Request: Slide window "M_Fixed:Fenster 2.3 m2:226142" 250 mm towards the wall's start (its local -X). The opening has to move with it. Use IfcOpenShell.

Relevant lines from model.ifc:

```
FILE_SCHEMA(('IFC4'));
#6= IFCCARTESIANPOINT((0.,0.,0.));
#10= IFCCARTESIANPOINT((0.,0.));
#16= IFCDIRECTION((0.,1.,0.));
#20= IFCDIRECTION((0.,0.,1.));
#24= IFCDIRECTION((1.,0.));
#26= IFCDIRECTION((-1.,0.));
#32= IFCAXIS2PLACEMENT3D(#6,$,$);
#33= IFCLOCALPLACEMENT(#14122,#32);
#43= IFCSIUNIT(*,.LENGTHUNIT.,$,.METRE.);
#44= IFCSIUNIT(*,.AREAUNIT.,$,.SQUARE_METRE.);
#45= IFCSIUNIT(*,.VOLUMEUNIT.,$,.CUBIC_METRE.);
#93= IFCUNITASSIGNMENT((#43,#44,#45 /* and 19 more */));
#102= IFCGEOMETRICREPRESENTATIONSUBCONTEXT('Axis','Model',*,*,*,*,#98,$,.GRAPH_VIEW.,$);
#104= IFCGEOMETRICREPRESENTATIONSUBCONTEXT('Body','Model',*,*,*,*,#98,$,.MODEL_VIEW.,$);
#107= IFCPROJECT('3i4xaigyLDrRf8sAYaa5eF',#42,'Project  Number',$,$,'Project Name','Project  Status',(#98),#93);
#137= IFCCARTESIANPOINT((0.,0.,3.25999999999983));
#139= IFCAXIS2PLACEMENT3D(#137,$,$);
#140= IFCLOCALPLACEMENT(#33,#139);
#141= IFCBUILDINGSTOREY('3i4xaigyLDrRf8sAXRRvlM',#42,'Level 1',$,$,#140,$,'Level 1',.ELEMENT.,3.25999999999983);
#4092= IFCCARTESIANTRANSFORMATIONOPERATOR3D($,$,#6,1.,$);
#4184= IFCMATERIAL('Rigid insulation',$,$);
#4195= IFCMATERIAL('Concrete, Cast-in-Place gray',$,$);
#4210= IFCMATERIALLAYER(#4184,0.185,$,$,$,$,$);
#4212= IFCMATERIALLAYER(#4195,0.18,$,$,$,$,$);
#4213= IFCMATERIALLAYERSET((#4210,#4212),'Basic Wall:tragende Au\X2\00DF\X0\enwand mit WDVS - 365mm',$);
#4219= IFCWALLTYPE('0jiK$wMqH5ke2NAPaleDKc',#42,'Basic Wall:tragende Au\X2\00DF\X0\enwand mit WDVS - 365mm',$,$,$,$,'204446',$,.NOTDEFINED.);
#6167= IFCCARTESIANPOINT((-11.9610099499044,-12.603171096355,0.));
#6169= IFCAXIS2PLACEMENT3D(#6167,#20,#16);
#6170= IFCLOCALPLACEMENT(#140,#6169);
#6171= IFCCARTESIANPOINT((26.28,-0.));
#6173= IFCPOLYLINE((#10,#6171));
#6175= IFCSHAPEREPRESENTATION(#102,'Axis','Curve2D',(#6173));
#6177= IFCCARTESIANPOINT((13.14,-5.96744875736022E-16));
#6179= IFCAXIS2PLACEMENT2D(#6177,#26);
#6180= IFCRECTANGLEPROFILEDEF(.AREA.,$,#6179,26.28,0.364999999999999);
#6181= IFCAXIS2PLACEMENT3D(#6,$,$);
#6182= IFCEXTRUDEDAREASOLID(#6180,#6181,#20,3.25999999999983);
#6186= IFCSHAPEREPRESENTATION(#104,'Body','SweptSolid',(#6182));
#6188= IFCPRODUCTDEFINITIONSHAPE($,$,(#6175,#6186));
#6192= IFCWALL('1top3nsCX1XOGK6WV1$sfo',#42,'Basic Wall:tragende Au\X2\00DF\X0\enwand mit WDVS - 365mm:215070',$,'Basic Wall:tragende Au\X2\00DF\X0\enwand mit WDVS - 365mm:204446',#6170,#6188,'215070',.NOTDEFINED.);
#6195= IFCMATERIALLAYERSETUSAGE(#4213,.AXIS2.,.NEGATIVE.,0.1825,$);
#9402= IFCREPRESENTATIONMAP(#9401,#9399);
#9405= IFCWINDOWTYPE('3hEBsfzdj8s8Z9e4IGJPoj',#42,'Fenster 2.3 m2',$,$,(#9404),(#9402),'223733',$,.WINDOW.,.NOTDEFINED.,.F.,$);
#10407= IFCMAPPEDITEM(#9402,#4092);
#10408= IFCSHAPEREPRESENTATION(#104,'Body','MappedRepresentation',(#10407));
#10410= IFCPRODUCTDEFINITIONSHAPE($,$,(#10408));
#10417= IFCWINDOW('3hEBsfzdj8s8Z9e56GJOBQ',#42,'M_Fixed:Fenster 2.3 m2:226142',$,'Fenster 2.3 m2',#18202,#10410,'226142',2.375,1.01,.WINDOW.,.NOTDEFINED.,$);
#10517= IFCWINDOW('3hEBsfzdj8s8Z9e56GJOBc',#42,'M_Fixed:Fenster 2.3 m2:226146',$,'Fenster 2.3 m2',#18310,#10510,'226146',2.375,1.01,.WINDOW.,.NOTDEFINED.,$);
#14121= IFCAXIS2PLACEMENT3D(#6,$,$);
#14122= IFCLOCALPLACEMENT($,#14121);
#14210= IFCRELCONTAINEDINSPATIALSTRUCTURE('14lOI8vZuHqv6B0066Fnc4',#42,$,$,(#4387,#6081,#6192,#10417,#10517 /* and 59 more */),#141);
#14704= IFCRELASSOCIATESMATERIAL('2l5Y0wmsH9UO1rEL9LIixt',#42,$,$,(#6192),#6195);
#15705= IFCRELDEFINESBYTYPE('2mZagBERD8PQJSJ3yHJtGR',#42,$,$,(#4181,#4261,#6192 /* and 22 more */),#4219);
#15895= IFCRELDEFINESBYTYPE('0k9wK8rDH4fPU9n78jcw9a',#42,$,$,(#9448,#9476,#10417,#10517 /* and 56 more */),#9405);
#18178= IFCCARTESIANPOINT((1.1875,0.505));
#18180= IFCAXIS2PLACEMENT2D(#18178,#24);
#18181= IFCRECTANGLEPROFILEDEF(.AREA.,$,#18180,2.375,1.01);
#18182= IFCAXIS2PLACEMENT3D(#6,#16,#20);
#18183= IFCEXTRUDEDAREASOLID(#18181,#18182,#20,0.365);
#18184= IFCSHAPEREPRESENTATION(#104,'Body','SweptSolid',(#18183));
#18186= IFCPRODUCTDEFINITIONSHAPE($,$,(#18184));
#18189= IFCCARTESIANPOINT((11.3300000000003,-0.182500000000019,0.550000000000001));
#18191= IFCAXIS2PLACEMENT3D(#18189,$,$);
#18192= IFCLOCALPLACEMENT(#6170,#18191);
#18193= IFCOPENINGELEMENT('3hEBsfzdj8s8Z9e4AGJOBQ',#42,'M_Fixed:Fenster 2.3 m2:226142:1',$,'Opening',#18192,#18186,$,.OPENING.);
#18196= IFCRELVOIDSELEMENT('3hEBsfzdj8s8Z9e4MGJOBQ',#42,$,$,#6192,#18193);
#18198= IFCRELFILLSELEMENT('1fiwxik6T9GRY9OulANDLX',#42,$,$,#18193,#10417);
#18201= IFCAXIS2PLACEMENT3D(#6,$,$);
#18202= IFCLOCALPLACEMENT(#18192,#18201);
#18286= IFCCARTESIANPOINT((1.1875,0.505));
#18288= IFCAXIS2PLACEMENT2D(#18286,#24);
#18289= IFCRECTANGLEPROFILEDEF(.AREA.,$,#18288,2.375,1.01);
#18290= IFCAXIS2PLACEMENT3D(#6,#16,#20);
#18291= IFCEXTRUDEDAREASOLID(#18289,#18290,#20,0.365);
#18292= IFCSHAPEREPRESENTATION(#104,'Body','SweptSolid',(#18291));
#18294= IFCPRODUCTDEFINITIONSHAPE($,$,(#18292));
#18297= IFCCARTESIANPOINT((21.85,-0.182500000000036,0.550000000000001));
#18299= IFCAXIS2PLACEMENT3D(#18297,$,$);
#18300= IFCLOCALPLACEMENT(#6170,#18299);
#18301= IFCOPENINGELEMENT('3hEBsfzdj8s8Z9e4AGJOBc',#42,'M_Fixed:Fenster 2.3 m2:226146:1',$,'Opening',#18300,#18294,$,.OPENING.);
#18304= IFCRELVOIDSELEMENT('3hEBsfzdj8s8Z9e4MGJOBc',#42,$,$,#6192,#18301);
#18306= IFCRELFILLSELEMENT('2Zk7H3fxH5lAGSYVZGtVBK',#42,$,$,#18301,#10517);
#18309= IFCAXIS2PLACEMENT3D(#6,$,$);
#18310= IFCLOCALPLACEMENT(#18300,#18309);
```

```python
import ifcopenshell
import ifcopenshell.api.geometry
import ifcopenshell.util.placement
import ifcopenshell.util.unit

model = ifcopenshell.open("model.ifc")
unit_scale = ifcopenshell.util.unit.calculate_unit_scale(model)

window = model.by_guid("3hEBsfzdj8s8Z9e56GJOBQ")
opening = window.FillsVoids[0].RelatingOpeningElement
wall = opening.VoidsElements[0].RelatingBuildingElement

wall_matrix = ifcopenshell.util.placement.get_local_placement(wall.ObjectPlacement)
shift = wall_matrix[:3, 0] * -0.25 / unit_scale
before = ifcopenshell.util.placement.get_local_placement(window.ObjectPlacement)[:3, 3].copy()

# The window is placed relative to its opening, so it follows when the opening moves.
matrix = ifcopenshell.util.placement.get_local_placement(opening.ObjectPlacement)
matrix[:3, 3] += shift
ifcopenshell.api.geometry.edit_object_placement(
    model, product=opening, matrix=matrix, is_si=False, should_transform_children=True
)

after = ifcopenshell.util.placement.get_local_placement(window.ObjectPlacement)[:3, 3]
print("window moved by", (after - before).round(3) + 0.0)

model.write("model_edited.ifc")
```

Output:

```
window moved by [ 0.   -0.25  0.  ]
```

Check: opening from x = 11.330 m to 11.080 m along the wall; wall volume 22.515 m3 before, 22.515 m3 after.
